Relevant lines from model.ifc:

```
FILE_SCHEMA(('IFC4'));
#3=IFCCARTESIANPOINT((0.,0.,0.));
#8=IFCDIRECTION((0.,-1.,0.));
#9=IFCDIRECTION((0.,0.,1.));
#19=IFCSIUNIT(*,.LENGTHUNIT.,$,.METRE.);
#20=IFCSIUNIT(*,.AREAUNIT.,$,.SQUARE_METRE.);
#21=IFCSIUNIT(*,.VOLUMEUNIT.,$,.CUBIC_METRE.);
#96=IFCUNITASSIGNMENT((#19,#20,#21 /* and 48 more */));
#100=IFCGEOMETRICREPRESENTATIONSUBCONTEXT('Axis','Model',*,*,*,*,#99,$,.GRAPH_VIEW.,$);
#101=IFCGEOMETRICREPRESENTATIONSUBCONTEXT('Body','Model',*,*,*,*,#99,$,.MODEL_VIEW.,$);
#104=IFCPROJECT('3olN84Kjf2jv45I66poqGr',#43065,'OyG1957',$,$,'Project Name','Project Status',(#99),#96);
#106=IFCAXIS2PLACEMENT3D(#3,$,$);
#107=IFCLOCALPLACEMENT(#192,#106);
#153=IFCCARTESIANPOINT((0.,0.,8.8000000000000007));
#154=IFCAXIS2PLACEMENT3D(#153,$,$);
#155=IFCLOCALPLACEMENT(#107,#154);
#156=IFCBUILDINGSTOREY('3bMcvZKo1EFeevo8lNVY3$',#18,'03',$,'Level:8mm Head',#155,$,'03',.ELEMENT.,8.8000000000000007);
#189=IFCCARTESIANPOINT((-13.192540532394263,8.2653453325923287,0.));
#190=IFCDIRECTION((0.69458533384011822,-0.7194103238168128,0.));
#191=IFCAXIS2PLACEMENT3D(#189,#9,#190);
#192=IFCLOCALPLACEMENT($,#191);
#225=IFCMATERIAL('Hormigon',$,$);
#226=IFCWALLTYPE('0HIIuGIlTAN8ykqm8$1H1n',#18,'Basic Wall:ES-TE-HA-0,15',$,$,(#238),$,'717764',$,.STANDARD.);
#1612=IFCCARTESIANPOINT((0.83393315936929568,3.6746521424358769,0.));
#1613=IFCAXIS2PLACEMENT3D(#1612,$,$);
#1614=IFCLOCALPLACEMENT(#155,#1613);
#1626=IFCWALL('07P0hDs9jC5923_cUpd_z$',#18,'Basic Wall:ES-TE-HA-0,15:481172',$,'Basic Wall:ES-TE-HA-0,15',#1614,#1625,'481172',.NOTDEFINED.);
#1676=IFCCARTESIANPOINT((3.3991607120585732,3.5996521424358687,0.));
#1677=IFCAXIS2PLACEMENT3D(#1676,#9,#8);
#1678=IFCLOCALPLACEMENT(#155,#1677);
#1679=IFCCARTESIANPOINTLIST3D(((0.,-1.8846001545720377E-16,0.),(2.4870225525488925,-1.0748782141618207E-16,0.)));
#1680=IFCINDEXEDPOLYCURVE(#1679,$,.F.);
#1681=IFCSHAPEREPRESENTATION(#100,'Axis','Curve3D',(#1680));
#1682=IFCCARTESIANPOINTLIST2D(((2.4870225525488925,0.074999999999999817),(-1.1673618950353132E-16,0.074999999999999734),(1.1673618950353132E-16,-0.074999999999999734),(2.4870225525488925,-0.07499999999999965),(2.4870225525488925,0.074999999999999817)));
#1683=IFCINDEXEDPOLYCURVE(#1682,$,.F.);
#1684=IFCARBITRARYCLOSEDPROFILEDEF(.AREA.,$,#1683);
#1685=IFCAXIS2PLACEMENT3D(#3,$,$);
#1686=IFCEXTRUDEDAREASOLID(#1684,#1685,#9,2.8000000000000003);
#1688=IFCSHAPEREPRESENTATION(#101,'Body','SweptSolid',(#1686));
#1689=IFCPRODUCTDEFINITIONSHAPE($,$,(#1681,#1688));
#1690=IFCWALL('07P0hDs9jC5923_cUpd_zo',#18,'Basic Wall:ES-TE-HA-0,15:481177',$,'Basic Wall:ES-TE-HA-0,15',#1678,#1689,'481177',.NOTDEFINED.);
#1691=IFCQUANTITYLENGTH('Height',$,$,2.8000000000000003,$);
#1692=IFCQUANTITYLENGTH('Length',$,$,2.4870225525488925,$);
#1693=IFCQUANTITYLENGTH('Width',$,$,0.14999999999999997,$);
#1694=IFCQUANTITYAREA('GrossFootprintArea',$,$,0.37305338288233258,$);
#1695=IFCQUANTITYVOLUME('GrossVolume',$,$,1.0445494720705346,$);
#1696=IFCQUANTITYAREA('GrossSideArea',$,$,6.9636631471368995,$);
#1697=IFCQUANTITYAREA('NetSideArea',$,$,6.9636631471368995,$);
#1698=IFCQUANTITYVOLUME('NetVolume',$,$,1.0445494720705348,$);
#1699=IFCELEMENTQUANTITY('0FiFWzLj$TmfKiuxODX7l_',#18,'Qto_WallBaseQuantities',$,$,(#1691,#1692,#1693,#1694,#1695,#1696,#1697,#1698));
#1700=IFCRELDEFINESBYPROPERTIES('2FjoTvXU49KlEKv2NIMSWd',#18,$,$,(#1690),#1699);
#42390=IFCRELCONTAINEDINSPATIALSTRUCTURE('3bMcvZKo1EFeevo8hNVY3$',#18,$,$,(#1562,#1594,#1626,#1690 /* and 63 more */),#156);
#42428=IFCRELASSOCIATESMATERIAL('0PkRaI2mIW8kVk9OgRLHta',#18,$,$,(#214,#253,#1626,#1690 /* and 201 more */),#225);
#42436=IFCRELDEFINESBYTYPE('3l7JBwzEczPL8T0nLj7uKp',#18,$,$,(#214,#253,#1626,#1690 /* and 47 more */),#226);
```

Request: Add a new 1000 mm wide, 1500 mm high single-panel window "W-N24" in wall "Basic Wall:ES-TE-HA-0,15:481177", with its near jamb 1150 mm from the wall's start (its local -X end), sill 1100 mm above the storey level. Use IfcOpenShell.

```python
import numpy as np
import ifcopenshell
import ifcopenshell.api.feature
import ifcopenshell.api.geometry
import ifcopenshell.api.pset
import ifcopenshell.api.root
import ifcopenshell.api.spatial
import ifcopenshell.geom
import ifcopenshell.util.element
import ifcopenshell.util.placement
import ifcopenshell.util.representation
import ifcopenshell.util.shape
import ifcopenshell.util.unit

model = ifcopenshell.open("model.ifc")
unit_scale = ifcopenshell.util.unit.calculate_unit_scale(model)
area_scale = ifcopenshell.util.unit.calculate_unit_scale(model, "AREAUNIT")
volume_scale = ifcopenshell.util.unit.calculate_unit_scale(model, "VOLUMEUNIT")
settings = ifcopenshell.geom.settings()


def volume(element):
    """Net volume in cubic metres, openings subtracted."""
    shape = ifcopenshell.geom.create_shape(settings, element)
    return ifcopenshell.util.shape.get_volume(shape.geometry)


wall = model.by_guid("07P0hDs9jC5923_cUpd_zo")
storey = ifcopenshell.util.element.get_container(wall, ifc_class="IfcBuildingStorey")
context = ifcopenshell.util.representation.get_context(model, "Model", "Body", "MODEL_VIEW")
before = volume(wall)

width, height, from_end, sill = 1, 1.5, 1.15, 1.1  # metres

# The wall runs along its own X axis, and the end named is its -X end.
wall_shape = ifcopenshell.geom.create_shape(settings, wall)
x, y, z = ifcopenshell.util.shape.get_vertices(wall_shape.geometry).T
start = x.min() + from_end
face, thickness = float(y.min()), float(y.max() - y.min())
wall_matrix = ifcopenshell.util.placement.get_local_placement(wall.ObjectPlacement)
level = ifcopenshell.util.placement.get_local_placement(storey.ObjectPlacement)[2, 3]


def in_wall(x, y):
    """Placement at x, y metres in the wall's axes, at sill height."""
    matrix = wall_matrix.copy()
    matrix[:, 3] = wall_matrix @ np.array([x / unit_scale, y / unit_scale, 0.0, 1.0])
    matrix[2, 3] = level + sill / unit_scale
    return matrix


# Opening: a box that overshoots both wall faces by 50 mm.
opening = ifcopenshell.api.root.create_entity(model, ifc_class="IfcOpeningElement", predefined_type="OPENING")
box = ifcopenshell.api.geometry.add_wall_representation(
    model, context=context, length=width, height=height, thickness=thickness + 0.1
)
ifcopenshell.api.geometry.assign_representation(model, product=opening, representation=box)
ifcopenshell.api.geometry.edit_object_placement(model, product=opening, matrix=in_wall(start, face - 0.05), is_si=False)
ifcopenshell.api.feature.add_feature(model, feature=opening, element=wall)

window = ifcopenshell.api.root.create_entity(model, ifc_class="IfcWindow", name="W-N24", predefined_type="WINDOW")
window.OverallWidth, window.OverallHeight = width / unit_scale, height / unit_scale
window.PartitioningType = "SINGLE_PANEL"
body = ifcopenshell.api.geometry.add_window_representation(
    model,
    context=context,
    overall_width=window.OverallWidth,
    overall_height=window.OverallHeight,
    partition_type="SINGLE_PANEL",
)
ifcopenshell.api.geometry.assign_representation(model, product=window, representation=body)
ifcopenshell.api.spatial.assign_container(model, products=[window], relating_structure=storey)
ifcopenshell.api.feature.add_filling(model, opening=opening, element=window)

# Centre the window in the wall's thickness.
ifcopenshell.api.geometry.edit_object_placement(model, product=window, matrix=in_wall(start, face), is_si=False)
window_shape = ifcopenshell.geom.create_shape(settings, window)
depth = ifcopenshell.util.shape.get_vertices(window_shape.geometry)[:, 1]
offset = face + thickness / 2 - (depth.min() + depth.max()) / 2
ifcopenshell.api.geometry.edit_object_placement(model, product=window, matrix=in_wall(start, offset), is_si=False)

after = volume(wall)

# Update the wall's stored quantities.
qto = model.by_id(ifcopenshell.util.element.get_pset(wall, "Qto_WallBaseQuantities", should_inherit=False)["id"])
ifcopenshell.api.pset.edit_qto(model, qto=qto, properties={
    "NetSideArea": after / thickness / area_scale,
    "NetVolume": after / volume_scale,
})

print(f"wall volume {before:.3f} -> {after:.3f} m3")

model.write("model_edited.ifc")
```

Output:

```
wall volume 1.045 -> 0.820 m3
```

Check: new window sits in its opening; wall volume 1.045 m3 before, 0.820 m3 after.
